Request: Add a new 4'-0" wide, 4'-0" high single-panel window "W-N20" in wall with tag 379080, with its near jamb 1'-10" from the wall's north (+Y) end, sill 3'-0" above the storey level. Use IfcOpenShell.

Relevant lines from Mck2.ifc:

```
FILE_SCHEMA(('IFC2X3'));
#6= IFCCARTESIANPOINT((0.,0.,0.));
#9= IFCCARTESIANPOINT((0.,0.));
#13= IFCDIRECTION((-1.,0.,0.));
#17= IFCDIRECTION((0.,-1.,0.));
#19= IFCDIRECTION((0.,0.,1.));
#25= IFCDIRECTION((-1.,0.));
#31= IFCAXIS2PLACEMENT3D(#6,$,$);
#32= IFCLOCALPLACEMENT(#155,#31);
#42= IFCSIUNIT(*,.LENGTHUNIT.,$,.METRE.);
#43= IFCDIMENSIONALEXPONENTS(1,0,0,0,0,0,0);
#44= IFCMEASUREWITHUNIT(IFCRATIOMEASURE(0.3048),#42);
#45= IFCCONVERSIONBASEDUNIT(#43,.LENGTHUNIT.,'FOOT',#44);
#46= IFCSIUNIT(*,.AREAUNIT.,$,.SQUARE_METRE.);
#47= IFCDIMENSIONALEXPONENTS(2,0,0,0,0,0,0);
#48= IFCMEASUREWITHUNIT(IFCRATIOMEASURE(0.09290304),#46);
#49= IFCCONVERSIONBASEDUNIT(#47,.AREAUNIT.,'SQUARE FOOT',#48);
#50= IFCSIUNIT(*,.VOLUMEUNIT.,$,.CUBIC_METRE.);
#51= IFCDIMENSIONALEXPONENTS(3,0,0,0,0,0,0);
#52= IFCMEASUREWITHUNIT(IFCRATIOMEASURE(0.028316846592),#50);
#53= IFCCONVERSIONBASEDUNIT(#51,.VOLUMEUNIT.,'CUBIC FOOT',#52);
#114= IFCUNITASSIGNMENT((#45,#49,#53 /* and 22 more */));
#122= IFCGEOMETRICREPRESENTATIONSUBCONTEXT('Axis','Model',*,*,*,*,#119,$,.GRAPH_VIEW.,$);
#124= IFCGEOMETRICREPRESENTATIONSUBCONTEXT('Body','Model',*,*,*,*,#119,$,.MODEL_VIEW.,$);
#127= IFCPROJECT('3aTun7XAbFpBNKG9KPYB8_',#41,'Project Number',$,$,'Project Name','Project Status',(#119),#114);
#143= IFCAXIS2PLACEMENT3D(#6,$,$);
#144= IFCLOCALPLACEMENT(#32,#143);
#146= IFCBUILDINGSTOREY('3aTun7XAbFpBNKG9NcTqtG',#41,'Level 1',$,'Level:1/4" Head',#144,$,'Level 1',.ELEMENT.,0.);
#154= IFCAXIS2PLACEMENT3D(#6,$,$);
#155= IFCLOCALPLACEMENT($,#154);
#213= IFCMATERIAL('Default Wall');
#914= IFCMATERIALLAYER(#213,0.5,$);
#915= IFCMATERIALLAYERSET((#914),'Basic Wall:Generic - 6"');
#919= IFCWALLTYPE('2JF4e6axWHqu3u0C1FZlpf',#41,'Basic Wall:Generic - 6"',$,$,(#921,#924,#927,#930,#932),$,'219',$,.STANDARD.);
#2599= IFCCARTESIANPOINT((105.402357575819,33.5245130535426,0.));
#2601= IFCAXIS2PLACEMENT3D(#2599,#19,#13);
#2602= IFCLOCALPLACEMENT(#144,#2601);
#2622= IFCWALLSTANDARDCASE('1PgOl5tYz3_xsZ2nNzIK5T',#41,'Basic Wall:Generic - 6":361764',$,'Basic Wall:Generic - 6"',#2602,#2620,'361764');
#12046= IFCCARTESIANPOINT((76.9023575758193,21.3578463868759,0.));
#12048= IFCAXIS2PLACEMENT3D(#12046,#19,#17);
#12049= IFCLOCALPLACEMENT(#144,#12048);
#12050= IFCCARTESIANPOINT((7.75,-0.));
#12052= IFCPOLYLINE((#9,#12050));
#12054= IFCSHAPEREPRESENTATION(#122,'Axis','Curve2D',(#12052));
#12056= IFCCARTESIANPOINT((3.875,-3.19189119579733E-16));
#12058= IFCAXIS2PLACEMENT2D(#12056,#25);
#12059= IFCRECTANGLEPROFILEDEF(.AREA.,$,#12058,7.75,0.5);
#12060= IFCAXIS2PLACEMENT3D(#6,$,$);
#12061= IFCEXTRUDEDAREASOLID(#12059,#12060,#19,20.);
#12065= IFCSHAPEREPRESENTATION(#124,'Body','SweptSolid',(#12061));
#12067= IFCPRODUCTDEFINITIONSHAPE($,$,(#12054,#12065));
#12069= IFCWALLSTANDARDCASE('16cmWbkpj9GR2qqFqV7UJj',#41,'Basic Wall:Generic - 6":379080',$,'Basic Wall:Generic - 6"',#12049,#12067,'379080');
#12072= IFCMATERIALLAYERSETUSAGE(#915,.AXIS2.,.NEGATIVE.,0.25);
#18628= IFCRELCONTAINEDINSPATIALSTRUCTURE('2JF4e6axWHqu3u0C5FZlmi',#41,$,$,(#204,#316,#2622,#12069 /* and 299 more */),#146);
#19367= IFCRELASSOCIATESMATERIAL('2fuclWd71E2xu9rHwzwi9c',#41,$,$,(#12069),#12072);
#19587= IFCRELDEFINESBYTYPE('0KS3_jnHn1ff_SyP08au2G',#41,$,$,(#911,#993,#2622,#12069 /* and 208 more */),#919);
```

```python
import numpy as np
import ifcopenshell
import ifcopenshell.api.feature
import ifcopenshell.api.geometry
import ifcopenshell.api.root
import ifcopenshell.api.spatial
import ifcopenshell.api.type
import ifcopenshell.geom
import ifcopenshell.util.element
import ifcopenshell.util.placement
import ifcopenshell.util.representation
import ifcopenshell.util.shape
import ifcopenshell.util.unit

model = ifcopenshell.open("Mck2.ifc")
unit_scale = ifcopenshell.util.unit.calculate_unit_scale(model)
settings = ifcopenshell.geom.settings()


def volume(element):
    """Net volume in cubic metres, openings subtracted."""
    shape = ifcopenshell.geom.create_shape(settings, element)
    return ifcopenshell.util.shape.get_volume(shape.geometry)


wall = model.by_guid("16cmWbkpj9GR2qqFqV7UJj")
storey = ifcopenshell.util.element.get_container(wall, ifc_class="IfcBuildingStorey")
context = ifcopenshell.util.representation.get_context(model, "Model", "Body", "MODEL_VIEW")
before = volume(wall)

width, height, from_end, sill = 1.2192, 1.2192, 0.5588, 0.9144  # metres

# The wall runs along its own X axis, and the end named is its -X end.
wall_shape = ifcopenshell.geom.create_shape(settings, wall)
x, y, z = ifcopenshell.util.shape.get_vertices(wall_shape.geometry).T
start = x.min() + from_end
face, thickness = float(y.min()), float(y.max() - y.min())
wall_matrix = ifcopenshell.util.placement.get_local_placement(wall.ObjectPlacement)
level = ifcopenshell.util.placement.get_local_placement(storey.ObjectPlacement)[2, 3]


def in_wall(x, y):
    """Placement at x, y metres in the wall's axes, at sill height."""
    matrix = wall_matrix.copy()
    matrix[:, 3] = wall_matrix @ np.array([x / unit_scale, y / unit_scale, 0.0, 1.0])
    matrix[2, 3] = level + sill / unit_scale
    return matrix


# Opening: a box that overshoots both wall faces by 50 mm.
opening = ifcopenshell.api.root.create_entity(model, ifc_class="IfcOpeningElement")
box = ifcopenshell.api.geometry.add_wall_representation(
    model, context=context, length=width, height=height, thickness=thickness + 0.1
)
ifcopenshell.api.geometry.assign_representation(model, product=opening, representation=box)
ifcopenshell.api.geometry.edit_object_placement(model, product=opening, matrix=in_wall(start, face - 0.05), is_si=False)
ifcopenshell.api.feature.add_feature(model, feature=opening, element=wall)

window = ifcopenshell.api.root.create_entity(model, ifc_class="IfcWindow", name="W-N20")
window.OverallWidth, window.OverallHeight = width / unit_scale, height / unit_scale
body = ifcopenshell.api.geometry.add_window_representation(
    model,
    context=context,
    overall_width=window.OverallWidth,
    overall_height=window.OverallHeight,
    partition_type="SINGLE_PANEL",
)
ifcopenshell.api.geometry.assign_representation(model, product=window, representation=body)
ifcopenshell.api.spatial.assign_container(model, products=[window], relating_structure=storey)
fills = ifcopenshell.api.feature.add_filling(model, opening=opening, element=window)
fills.OwnerHistory = window.OwnerHistory  # required in IFC2X3

# IFC2X3 keeps the operation on the window style.
style = ifcopenshell.api.root.create_entity(model, ifc_class="IfcWindowStyle", name="W-N20")
style.OperationType, style.ConstructionType = "SINGLE_PANEL", "NOTDEFINED"
style.ParameterTakesPrecedence = style.Sizeable = False
ifcopenshell.api.type.assign_type(model, related_objects=[window], relating_type=style)

# Centre the window in the wall's thickness.
ifcopenshell.api.geometry.edit_object_placement(model, product=window, matrix=in_wall(start, face), is_si=False)
window_shape = ifcopenshell.geom.create_shape(settings, window)
depth = ifcopenshell.util.shape.get_vertices(window_shape.geometry)[:, 1]
offset = face + thickness / 2 - (depth.min() + depth.max()) / 2
ifcopenshell.api.geometry.edit_object_placement(model, product=window, matrix=in_wall(start, offset), is_si=False)

after = volume(wall)

print(f"wall volume {before:.3f} -> {after:.3f} m3")

model.write("Mck2-out.ifc")
```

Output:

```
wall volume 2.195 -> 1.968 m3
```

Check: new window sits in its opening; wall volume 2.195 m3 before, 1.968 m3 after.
